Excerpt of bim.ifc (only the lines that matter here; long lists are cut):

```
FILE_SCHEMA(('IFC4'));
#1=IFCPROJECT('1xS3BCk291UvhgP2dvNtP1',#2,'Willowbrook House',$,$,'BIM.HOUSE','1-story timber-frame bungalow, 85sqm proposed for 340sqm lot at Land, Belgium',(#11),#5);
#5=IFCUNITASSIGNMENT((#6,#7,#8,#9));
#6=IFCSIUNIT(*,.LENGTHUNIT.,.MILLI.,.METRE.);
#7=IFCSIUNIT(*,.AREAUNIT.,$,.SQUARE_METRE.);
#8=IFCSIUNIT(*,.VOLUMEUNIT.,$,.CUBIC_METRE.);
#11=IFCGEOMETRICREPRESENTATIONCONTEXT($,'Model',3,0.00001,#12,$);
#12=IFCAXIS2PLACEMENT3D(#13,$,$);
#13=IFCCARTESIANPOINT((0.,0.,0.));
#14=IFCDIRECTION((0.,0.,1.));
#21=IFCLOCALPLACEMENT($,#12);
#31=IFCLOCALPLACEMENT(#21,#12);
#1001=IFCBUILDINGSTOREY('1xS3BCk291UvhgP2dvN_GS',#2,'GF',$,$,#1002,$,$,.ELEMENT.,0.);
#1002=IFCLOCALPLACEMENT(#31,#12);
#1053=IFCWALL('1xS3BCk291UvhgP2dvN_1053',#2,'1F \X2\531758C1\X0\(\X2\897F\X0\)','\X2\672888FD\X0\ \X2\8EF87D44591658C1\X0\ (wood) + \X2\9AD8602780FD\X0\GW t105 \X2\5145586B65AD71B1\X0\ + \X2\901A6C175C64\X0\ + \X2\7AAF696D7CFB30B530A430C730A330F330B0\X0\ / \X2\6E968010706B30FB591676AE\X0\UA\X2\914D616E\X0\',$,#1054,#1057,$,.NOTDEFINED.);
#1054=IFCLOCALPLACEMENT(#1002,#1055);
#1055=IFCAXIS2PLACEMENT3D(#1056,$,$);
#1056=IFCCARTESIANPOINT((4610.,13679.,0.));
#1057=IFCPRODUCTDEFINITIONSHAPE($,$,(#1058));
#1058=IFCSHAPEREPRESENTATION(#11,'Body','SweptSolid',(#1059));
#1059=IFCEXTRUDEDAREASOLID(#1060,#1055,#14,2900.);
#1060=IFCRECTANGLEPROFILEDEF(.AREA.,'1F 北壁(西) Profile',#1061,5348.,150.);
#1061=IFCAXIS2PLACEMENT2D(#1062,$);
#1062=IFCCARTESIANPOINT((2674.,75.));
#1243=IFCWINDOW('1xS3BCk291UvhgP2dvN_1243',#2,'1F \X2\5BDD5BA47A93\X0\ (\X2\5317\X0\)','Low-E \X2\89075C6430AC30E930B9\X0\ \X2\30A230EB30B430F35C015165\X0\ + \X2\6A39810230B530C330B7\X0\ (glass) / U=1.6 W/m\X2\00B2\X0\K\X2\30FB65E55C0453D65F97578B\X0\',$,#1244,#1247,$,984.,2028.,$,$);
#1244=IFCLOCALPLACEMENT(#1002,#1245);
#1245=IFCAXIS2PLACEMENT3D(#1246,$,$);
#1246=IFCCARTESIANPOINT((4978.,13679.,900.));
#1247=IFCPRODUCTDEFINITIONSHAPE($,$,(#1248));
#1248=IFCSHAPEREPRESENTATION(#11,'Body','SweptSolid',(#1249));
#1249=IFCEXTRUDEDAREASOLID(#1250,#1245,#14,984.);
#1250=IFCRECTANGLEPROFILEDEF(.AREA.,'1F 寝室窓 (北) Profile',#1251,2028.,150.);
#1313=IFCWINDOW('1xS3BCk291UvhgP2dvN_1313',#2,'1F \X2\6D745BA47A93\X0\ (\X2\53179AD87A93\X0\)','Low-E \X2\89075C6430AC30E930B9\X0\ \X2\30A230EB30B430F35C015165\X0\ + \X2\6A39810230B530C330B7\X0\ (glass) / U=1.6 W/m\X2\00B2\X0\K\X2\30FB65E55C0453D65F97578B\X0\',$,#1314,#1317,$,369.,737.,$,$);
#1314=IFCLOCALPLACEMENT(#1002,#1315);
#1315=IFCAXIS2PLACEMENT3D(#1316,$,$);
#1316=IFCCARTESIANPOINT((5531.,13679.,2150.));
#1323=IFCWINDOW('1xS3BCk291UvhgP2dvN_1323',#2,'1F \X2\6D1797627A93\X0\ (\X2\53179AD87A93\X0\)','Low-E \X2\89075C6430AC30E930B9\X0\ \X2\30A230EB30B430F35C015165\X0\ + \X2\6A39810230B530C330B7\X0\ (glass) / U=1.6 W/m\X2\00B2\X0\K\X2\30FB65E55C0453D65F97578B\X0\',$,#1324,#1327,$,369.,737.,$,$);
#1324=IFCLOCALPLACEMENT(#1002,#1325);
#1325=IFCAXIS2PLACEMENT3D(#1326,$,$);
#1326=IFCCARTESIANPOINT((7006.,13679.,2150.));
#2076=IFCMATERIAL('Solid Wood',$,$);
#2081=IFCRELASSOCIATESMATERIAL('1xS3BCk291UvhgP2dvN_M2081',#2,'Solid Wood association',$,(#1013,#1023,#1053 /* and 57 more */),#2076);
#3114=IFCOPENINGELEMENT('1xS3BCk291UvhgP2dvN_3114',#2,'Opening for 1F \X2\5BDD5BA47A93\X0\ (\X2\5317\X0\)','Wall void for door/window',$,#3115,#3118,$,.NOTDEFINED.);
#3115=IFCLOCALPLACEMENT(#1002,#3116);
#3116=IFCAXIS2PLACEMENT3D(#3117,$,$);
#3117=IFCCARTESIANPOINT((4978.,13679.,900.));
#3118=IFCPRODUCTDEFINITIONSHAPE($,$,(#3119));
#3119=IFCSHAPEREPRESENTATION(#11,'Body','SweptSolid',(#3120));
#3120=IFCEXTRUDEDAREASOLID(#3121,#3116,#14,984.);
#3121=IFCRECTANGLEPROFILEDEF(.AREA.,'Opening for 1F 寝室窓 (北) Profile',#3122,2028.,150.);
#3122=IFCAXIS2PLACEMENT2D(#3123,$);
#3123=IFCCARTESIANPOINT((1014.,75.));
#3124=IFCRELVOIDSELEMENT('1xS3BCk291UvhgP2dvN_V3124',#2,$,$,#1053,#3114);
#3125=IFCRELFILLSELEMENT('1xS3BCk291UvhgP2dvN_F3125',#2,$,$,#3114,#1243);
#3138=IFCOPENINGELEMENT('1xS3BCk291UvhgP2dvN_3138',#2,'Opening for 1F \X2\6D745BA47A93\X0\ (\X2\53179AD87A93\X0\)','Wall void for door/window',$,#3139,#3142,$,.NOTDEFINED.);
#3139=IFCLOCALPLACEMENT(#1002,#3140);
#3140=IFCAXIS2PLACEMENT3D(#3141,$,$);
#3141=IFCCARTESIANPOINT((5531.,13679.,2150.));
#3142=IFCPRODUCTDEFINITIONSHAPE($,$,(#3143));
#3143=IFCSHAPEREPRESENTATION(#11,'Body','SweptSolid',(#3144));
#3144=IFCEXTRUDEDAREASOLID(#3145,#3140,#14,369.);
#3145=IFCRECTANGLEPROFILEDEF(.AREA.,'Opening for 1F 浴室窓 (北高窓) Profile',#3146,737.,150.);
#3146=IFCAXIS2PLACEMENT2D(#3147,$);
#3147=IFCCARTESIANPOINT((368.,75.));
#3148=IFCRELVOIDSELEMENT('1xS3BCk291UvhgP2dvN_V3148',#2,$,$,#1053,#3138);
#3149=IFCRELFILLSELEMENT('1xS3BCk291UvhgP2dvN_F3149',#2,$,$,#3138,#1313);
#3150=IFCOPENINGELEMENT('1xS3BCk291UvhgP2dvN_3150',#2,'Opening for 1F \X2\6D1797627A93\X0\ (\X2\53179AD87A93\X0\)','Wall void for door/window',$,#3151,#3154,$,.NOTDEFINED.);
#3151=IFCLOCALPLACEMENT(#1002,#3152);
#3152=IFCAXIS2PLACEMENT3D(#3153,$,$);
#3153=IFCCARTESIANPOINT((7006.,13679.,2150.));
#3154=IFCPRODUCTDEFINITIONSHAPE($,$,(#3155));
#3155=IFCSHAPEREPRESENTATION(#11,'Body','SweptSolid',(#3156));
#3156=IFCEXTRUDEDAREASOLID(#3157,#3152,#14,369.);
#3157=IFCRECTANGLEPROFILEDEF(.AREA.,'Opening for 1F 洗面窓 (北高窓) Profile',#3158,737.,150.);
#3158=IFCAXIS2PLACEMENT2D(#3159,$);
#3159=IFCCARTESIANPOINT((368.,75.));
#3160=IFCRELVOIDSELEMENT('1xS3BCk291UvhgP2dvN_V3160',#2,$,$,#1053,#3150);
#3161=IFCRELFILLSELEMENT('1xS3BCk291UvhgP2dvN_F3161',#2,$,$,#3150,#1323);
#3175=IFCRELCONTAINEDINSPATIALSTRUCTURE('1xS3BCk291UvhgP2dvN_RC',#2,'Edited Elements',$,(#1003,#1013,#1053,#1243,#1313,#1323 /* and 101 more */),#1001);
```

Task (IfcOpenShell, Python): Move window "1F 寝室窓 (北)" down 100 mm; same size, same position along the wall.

```python
import numpy as np
import ifcopenshell
import ifcopenshell.api.geometry
import ifcopenshell.util.placement
import ifcopenshell.util.unit

model = ifcopenshell.open("bim.ifc")
unit_scale = ifcopenshell.util.unit.calculate_unit_scale(model)

window = model.by_id(1243)
opening = window.FillsVoids[0].RelatingOpeningElement
dz = -0.1 / unit_scale

shift = np.array([0.0, 0.0, dz])
# The window is not placed relative to its opening, so move both.
for product in (opening, window):
    matrix = ifcopenshell.util.placement.get_local_placement(product.ObjectPlacement)
    matrix[:3, 3] += shift
    ifcopenshell.api.geometry.edit_object_placement(model, product=product, matrix=matrix, is_si=False)

print(f"moved by {dz * unit_scale:+.3f} m")

model.write("bim_v2.ifc")
```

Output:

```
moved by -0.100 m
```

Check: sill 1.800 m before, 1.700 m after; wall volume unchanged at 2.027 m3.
